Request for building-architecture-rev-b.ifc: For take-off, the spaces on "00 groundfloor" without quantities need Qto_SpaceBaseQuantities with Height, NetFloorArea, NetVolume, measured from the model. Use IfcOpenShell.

First a look at what the model holds.

```python
import ifcopenshell
import ifcopenshell.util.element
import ifcopenshell.util.unit

model = ifcopenshell.open("building-architecture-rev-b.ifc")
print(model.schema)
for unit_type in ("LENGTHUNIT", "AREAUNIT", "VOLUMEUNIT"):
    print(unit_type, ifcopenshell.util.unit.calculate_unit_scale(model, unit_type))
storey = next(s for s in model.by_type("IfcBuildingStorey") if s.Name == "00 groundfloor")
spaces = [e for e in ifcopenshell.util.element.get_decomposition(storey) if e.is_a("IfcSpace")]
for e in sorted(spaces, key=lambda e: e.id()):
    print(e.id(), e.is_a(), e.Name, list(ifcopenshell.util.element.get_psets(e, qtos_only=True)), sep=" | ")
```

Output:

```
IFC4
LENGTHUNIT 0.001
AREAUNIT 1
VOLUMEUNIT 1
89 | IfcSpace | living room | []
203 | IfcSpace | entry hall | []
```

```python
import ifcopenshell
import ifcopenshell.api.pset
import ifcopenshell.geom
import ifcopenshell.util.element
import ifcopenshell.util.shape
import ifcopenshell.util.unit

model = ifcopenshell.open("building-architecture-rev-b.ifc")
unit_scale = ifcopenshell.util.unit.calculate_unit_scale(model)
area_scale = ifcopenshell.util.unit.calculate_unit_scale(model, "AREAUNIT")
volume_scale = ifcopenshell.util.unit.calculate_unit_scale(model, "VOLUMEUNIT")
settings = ifcopenshell.geom.settings()

storey = next(s for s in model.by_type("IfcBuildingStorey") if s.Name == "00 groundfloor")
spaces = [e for e in ifcopenshell.util.element.get_decomposition(storey) if e.is_a("IfcSpace")]

for e in sorted(spaces, key=lambda e: e.id()):
    if ifcopenshell.util.element.get_psets(e, qtos_only=True, should_inherit=False):
        continue
    # Geometry comes back in metres, in the element's own axes.
    shape = ifcopenshell.geom.create_shape(settings, e)
    values = {
        "Height": ifcopenshell.util.shape.get_z(shape.geometry) / unit_scale,
        "NetFloorArea": ifcopenshell.util.shape.get_footprint_area(shape.geometry) / area_scale,
        "NetVolume": ifcopenshell.util.shape.get_volume(shape.geometry) / volume_scale,
    }
    qto = ifcopenshell.api.pset.add_qto(model, product=e, name="Qto_SpaceBaseQuantities")
    ifcopenshell.api.pset.edit_qto(model, qto=qto, properties=values)
    print(e.id(), {k: round(v, 3) for k, v in values.items()})

model.write("building-architecture-rev-b_rev.ifc")
```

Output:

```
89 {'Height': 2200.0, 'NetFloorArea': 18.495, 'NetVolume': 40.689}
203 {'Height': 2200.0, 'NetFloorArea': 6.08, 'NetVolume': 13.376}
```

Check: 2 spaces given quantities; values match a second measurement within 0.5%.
